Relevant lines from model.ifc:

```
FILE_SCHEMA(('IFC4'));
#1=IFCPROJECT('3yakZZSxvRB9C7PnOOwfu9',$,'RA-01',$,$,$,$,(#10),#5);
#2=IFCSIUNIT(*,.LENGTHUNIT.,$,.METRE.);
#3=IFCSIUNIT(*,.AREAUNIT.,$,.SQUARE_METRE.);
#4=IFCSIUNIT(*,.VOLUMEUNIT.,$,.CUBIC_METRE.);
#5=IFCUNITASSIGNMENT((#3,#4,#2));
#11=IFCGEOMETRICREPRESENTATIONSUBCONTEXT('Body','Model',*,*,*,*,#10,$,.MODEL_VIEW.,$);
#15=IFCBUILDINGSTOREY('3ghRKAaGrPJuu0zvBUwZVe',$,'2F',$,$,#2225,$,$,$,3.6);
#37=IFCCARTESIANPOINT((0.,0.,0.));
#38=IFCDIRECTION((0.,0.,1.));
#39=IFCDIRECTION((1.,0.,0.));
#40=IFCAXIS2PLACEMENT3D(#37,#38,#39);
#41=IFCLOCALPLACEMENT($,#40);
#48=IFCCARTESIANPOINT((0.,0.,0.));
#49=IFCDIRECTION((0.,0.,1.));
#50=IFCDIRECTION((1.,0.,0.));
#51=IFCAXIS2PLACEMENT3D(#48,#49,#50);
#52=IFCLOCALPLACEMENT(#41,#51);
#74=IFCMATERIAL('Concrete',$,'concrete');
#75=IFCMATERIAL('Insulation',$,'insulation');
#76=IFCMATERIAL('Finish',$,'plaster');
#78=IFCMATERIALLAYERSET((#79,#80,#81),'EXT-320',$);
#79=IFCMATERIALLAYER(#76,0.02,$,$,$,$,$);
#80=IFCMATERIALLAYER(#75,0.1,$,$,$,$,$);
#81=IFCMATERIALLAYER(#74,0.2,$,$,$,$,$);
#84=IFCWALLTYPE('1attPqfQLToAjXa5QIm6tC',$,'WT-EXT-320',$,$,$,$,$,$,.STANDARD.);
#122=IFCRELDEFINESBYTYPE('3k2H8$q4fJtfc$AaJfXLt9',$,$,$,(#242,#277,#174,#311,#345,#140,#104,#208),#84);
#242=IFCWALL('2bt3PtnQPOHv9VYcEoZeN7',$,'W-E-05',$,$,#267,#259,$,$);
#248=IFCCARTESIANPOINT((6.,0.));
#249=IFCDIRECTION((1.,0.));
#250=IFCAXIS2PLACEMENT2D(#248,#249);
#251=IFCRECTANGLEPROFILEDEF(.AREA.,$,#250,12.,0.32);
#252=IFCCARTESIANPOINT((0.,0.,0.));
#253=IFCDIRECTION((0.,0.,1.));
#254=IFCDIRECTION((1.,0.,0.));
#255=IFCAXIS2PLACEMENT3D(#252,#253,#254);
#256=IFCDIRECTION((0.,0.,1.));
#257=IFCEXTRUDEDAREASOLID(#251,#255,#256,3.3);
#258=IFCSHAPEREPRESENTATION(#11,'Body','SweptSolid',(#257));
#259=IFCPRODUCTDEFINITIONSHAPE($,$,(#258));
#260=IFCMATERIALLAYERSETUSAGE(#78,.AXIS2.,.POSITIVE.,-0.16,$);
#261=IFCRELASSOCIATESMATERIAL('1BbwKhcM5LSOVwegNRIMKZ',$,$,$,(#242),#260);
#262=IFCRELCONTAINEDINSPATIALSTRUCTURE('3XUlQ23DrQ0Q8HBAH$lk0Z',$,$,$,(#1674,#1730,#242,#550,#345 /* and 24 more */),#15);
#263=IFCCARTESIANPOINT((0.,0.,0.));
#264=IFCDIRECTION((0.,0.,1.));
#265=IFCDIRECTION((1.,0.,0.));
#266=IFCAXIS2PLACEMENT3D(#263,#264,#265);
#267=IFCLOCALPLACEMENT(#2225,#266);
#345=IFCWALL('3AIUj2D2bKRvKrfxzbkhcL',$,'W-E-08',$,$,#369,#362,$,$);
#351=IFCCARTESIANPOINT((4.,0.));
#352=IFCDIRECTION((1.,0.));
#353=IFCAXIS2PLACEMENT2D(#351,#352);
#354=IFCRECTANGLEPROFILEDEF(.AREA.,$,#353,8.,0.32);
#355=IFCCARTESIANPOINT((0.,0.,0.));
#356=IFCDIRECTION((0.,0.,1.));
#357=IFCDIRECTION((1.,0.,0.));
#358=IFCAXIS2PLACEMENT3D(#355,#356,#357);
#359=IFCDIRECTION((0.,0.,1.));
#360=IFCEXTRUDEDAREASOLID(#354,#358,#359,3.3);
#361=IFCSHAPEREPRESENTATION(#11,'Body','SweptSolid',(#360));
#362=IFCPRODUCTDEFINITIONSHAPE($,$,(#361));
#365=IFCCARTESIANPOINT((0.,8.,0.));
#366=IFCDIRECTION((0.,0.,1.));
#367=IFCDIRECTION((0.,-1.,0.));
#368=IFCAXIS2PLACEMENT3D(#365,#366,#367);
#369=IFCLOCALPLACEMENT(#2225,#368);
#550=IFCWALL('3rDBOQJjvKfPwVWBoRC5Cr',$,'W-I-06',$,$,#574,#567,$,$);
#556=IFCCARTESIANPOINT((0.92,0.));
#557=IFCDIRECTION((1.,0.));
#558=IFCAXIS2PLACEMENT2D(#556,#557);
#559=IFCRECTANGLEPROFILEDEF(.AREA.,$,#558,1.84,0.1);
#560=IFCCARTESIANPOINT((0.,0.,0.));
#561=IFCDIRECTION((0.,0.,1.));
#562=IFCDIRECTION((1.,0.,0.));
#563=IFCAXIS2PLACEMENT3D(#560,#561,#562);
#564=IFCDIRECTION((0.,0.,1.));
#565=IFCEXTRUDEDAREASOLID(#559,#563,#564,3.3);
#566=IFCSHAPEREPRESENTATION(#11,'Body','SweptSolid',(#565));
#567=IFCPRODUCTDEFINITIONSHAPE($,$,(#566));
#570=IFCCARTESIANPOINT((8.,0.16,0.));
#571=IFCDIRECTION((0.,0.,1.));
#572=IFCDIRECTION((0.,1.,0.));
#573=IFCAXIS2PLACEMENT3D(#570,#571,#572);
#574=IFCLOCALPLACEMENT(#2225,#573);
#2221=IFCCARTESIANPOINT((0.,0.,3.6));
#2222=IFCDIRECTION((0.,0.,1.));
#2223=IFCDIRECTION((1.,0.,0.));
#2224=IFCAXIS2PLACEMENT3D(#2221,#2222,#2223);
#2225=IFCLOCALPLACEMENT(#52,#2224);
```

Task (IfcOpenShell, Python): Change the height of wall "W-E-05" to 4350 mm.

```python
import ifcopenshell
import ifcopenshell.geom
import ifcopenshell.util.representation
import ifcopenshell.util.shape
import ifcopenshell.util.unit

model = ifcopenshell.open("model.ifc")
unit_scale = ifcopenshell.util.unit.calculate_unit_scale(model)
settings = ifcopenshell.geom.settings()


def volume(element):
    """Net volume in cubic metres, openings subtracted."""
    shape = ifcopenshell.geom.create_shape(settings, element)
    return ifcopenshell.util.shape.get_volume(shape.geometry)


wall = model.by_guid("2bt3PtnQPOHv9VYcEoZeN7")
before = volume(wall)

body = ifcopenshell.util.representation.get_representation(wall, "Model", "Body")
solid = body.Items[0]
old_height = solid.Depth
solid.Depth = 4.35 / unit_scale
after = volume(wall)

print(f"height {old_height:g} -> {solid.Depth:g}, volume {before:.3f} -> {after:.3f} m3")

model.write("model_v2.ifc")
```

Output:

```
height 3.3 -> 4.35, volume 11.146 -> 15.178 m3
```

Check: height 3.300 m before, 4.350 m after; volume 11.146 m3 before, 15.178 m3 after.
